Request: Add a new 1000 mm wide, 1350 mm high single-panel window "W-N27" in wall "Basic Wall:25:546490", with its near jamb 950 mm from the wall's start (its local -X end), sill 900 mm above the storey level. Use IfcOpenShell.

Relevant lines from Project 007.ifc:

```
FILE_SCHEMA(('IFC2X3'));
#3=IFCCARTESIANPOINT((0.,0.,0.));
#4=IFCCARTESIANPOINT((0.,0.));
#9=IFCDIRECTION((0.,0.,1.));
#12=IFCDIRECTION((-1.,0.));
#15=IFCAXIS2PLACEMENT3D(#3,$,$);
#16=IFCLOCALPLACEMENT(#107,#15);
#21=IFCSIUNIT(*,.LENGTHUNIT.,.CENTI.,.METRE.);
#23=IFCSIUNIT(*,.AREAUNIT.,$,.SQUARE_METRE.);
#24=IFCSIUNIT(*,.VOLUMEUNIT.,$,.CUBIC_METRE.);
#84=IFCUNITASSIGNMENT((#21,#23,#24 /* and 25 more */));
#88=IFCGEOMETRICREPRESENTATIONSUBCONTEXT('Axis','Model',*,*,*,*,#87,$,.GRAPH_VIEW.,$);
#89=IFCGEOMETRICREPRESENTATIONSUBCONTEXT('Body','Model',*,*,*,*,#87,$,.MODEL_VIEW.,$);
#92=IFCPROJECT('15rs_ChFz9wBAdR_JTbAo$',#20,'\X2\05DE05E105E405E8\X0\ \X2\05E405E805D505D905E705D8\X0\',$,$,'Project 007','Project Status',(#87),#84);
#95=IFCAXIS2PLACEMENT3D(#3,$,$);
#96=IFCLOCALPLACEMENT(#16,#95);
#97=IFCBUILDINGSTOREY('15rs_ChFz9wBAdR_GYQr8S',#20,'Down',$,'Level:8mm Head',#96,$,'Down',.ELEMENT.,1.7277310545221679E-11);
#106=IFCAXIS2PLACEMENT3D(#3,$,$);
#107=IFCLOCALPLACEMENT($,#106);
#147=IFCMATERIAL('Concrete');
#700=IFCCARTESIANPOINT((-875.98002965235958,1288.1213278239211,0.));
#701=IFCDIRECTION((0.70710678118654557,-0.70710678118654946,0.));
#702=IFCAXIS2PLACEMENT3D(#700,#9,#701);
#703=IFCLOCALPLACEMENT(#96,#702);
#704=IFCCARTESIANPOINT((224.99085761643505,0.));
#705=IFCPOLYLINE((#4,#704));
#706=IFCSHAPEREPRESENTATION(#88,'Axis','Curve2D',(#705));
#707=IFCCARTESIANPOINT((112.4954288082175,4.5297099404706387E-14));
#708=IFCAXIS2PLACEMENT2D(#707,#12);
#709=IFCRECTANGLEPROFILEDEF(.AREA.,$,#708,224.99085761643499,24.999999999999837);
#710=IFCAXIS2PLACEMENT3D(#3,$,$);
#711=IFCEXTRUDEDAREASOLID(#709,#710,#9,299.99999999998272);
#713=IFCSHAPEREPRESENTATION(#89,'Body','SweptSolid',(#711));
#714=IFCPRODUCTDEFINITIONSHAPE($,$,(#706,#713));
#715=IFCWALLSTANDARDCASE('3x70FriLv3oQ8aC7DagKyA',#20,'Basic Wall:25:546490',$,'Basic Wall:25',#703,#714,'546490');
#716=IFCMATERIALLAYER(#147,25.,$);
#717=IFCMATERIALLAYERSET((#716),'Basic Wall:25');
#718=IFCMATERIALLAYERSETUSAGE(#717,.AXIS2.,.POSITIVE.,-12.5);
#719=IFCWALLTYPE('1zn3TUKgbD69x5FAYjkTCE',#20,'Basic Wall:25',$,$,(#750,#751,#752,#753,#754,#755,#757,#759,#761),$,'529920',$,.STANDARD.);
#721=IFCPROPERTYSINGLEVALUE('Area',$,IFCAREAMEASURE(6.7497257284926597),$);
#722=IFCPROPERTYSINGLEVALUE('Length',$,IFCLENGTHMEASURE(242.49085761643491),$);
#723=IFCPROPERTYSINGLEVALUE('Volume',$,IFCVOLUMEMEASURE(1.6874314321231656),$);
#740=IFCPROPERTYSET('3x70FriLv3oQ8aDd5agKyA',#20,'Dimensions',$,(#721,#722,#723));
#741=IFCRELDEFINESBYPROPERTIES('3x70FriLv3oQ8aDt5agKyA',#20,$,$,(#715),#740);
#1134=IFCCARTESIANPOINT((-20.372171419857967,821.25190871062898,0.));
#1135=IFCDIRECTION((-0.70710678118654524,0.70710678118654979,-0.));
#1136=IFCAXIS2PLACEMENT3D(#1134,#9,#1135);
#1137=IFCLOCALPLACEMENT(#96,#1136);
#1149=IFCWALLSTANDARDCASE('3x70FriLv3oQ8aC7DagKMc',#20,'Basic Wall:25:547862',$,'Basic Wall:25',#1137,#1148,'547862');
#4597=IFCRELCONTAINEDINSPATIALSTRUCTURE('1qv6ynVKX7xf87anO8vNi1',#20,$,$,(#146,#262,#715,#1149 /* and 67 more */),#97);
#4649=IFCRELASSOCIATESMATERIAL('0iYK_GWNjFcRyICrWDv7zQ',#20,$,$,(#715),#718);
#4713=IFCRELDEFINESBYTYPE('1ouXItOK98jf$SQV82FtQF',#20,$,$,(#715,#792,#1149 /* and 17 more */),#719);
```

```python
import numpy as np
import ifcopenshell
import ifcopenshell.api.feature
import ifcopenshell.api.geometry
import ifcopenshell.api.pset
import ifcopenshell.api.root
import ifcopenshell.api.spatial
import ifcopenshell.api.type
import ifcopenshell.geom
import ifcopenshell.util.element
import ifcopenshell.util.placement
import ifcopenshell.util.representation
import ifcopenshell.util.shape
import ifcopenshell.util.unit

model = ifcopenshell.open("Project 007.ifc")
unit_scale = ifcopenshell.util.unit.calculate_unit_scale(model)
area_scale = ifcopenshell.util.unit.calculate_unit_scale(model, "AREAUNIT")
volume_scale = ifcopenshell.util.unit.calculate_unit_scale(model, "VOLUMEUNIT")
settings = ifcopenshell.geom.settings()


def volume(element):
    """Net volume in cubic metres, openings subtracted."""
    shape = ifcopenshell.geom.create_shape(settings, element)
    return ifcopenshell.util.shape.get_volume(shape.geometry)


wall = model.by_id(715)
storey = ifcopenshell.util.element.get_container(wall, ifc_class="IfcBuildingStorey")
context = ifcopenshell.util.representation.get_context(model, "Model", "Body", "MODEL_VIEW")
before = volume(wall)

width, height, from_end, sill = 1, 1.35, 0.95, 0.9  # metres

# The wall runs along its own X axis, and the end named is its -X end.
wall_shape = ifcopenshell.geom.create_shape(settings, wall)
x, y, z = ifcopenshell.util.shape.get_vertices(wall_shape.geometry).T
start = x.min() + from_end
face, thickness = float(y.min()), float(y.max() - y.min())
wall_matrix = ifcopenshell.util.placement.get_local_placement(wall.ObjectPlacement)
level = ifcopenshell.util.placement.get_local_placement(storey.ObjectPlacement)[2, 3]


def in_wall(x, y):
    """Placement at x, y metres in the wall's axes, at sill height."""
    matrix = wall_matrix.copy()
    matrix[:, 3] = wall_matrix @ np.array([x / unit_scale, y / unit_scale, 0.0, 1.0])
    matrix[2, 3] = level + sill / unit_scale
    return matrix


# Opening: a box that overshoots both wall faces by 50 mm.
opening = ifcopenshell.api.root.create_entity(model, ifc_class="IfcOpeningElement")
box = ifcopenshell.api.geometry.add_wall_representation(
    model, context=context, length=width, height=height, thickness=thickness + 0.1
)
ifcopenshell.api.geometry.assign_representation(model, product=opening, representation=box)
ifcopenshell.api.geometry.edit_object_placement(model, product=opening, matrix=in_wall(start, face - 0.05), is_si=False)
ifcopenshell.api.feature.add_feature(model, feature=opening, element=wall)

window = ifcopenshell.api.root.create_entity(model, ifc_class="IfcWindow", name="W-N27")
window.OverallWidth, window.OverallHeight = width / unit_scale, height / unit_scale
body = ifcopenshell.api.geometry.add_window_representation(
    model,
    context=context,
    overall_width=window.OverallWidth,
    overall_height=window.OverallHeight,
    partition_type="SINGLE_PANEL",
)
ifcopenshell.api.geometry.assign_representation(model, product=window, representation=body)
ifcopenshell.api.spatial.assign_container(model, products=[window], relating_structure=storey)
fills = ifcopenshell.api.feature.add_filling(model, opening=opening, element=window)
fills.OwnerHistory = window.OwnerHistory  # required in IFC2X3

# IFC2X3 keeps the operation on the window style.
style = ifcopenshell.api.root.create_entity(model, ifc_class="IfcWindowStyle", name="W-N27")
style.OperationType, style.ConstructionType = "SINGLE_PANEL", "NOTDEFINED"
style.ParameterTakesPrecedence = style.Sizeable = False
ifcopenshell.api.type.assign_type(model, related_objects=[window], relating_type=style)

# Centre the window in the wall's thickness.
ifcopenshell.api.geometry.edit_object_placement(model, product=window, matrix=in_wall(start, face), is_si=False)
window_shape = ifcopenshell.geom.create_shape(settings, window)
depth = ifcopenshell.util.shape.get_vertices(window_shape.geometry)[:, 1]
offset = face + thickness / 2 - (depth.min() + depth.max()) / 2
ifcopenshell.api.geometry.edit_object_placement(model, product=window, matrix=in_wall(start, offset), is_si=False)

after = volume(wall)

# Update the wall's stored quantities.
pset = model.by_id(ifcopenshell.util.element.get_pset(wall, "Dimensions", should_inherit=False)["id"])
ifcopenshell.api.pset.edit_pset(model, pset=pset, properties={
    "Area": model.create_entity("IfcAreaMeasure", after / thickness / area_scale),
    "Volume": model.create_entity("IfcVolumeMeasure", after / volume_scale),
})

print(f"wall volume {before:.3f} -> {after:.3f} m3")

model.write("Project 007_rev.ifc")
```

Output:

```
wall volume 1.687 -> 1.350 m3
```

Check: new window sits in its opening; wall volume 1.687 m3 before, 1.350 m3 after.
